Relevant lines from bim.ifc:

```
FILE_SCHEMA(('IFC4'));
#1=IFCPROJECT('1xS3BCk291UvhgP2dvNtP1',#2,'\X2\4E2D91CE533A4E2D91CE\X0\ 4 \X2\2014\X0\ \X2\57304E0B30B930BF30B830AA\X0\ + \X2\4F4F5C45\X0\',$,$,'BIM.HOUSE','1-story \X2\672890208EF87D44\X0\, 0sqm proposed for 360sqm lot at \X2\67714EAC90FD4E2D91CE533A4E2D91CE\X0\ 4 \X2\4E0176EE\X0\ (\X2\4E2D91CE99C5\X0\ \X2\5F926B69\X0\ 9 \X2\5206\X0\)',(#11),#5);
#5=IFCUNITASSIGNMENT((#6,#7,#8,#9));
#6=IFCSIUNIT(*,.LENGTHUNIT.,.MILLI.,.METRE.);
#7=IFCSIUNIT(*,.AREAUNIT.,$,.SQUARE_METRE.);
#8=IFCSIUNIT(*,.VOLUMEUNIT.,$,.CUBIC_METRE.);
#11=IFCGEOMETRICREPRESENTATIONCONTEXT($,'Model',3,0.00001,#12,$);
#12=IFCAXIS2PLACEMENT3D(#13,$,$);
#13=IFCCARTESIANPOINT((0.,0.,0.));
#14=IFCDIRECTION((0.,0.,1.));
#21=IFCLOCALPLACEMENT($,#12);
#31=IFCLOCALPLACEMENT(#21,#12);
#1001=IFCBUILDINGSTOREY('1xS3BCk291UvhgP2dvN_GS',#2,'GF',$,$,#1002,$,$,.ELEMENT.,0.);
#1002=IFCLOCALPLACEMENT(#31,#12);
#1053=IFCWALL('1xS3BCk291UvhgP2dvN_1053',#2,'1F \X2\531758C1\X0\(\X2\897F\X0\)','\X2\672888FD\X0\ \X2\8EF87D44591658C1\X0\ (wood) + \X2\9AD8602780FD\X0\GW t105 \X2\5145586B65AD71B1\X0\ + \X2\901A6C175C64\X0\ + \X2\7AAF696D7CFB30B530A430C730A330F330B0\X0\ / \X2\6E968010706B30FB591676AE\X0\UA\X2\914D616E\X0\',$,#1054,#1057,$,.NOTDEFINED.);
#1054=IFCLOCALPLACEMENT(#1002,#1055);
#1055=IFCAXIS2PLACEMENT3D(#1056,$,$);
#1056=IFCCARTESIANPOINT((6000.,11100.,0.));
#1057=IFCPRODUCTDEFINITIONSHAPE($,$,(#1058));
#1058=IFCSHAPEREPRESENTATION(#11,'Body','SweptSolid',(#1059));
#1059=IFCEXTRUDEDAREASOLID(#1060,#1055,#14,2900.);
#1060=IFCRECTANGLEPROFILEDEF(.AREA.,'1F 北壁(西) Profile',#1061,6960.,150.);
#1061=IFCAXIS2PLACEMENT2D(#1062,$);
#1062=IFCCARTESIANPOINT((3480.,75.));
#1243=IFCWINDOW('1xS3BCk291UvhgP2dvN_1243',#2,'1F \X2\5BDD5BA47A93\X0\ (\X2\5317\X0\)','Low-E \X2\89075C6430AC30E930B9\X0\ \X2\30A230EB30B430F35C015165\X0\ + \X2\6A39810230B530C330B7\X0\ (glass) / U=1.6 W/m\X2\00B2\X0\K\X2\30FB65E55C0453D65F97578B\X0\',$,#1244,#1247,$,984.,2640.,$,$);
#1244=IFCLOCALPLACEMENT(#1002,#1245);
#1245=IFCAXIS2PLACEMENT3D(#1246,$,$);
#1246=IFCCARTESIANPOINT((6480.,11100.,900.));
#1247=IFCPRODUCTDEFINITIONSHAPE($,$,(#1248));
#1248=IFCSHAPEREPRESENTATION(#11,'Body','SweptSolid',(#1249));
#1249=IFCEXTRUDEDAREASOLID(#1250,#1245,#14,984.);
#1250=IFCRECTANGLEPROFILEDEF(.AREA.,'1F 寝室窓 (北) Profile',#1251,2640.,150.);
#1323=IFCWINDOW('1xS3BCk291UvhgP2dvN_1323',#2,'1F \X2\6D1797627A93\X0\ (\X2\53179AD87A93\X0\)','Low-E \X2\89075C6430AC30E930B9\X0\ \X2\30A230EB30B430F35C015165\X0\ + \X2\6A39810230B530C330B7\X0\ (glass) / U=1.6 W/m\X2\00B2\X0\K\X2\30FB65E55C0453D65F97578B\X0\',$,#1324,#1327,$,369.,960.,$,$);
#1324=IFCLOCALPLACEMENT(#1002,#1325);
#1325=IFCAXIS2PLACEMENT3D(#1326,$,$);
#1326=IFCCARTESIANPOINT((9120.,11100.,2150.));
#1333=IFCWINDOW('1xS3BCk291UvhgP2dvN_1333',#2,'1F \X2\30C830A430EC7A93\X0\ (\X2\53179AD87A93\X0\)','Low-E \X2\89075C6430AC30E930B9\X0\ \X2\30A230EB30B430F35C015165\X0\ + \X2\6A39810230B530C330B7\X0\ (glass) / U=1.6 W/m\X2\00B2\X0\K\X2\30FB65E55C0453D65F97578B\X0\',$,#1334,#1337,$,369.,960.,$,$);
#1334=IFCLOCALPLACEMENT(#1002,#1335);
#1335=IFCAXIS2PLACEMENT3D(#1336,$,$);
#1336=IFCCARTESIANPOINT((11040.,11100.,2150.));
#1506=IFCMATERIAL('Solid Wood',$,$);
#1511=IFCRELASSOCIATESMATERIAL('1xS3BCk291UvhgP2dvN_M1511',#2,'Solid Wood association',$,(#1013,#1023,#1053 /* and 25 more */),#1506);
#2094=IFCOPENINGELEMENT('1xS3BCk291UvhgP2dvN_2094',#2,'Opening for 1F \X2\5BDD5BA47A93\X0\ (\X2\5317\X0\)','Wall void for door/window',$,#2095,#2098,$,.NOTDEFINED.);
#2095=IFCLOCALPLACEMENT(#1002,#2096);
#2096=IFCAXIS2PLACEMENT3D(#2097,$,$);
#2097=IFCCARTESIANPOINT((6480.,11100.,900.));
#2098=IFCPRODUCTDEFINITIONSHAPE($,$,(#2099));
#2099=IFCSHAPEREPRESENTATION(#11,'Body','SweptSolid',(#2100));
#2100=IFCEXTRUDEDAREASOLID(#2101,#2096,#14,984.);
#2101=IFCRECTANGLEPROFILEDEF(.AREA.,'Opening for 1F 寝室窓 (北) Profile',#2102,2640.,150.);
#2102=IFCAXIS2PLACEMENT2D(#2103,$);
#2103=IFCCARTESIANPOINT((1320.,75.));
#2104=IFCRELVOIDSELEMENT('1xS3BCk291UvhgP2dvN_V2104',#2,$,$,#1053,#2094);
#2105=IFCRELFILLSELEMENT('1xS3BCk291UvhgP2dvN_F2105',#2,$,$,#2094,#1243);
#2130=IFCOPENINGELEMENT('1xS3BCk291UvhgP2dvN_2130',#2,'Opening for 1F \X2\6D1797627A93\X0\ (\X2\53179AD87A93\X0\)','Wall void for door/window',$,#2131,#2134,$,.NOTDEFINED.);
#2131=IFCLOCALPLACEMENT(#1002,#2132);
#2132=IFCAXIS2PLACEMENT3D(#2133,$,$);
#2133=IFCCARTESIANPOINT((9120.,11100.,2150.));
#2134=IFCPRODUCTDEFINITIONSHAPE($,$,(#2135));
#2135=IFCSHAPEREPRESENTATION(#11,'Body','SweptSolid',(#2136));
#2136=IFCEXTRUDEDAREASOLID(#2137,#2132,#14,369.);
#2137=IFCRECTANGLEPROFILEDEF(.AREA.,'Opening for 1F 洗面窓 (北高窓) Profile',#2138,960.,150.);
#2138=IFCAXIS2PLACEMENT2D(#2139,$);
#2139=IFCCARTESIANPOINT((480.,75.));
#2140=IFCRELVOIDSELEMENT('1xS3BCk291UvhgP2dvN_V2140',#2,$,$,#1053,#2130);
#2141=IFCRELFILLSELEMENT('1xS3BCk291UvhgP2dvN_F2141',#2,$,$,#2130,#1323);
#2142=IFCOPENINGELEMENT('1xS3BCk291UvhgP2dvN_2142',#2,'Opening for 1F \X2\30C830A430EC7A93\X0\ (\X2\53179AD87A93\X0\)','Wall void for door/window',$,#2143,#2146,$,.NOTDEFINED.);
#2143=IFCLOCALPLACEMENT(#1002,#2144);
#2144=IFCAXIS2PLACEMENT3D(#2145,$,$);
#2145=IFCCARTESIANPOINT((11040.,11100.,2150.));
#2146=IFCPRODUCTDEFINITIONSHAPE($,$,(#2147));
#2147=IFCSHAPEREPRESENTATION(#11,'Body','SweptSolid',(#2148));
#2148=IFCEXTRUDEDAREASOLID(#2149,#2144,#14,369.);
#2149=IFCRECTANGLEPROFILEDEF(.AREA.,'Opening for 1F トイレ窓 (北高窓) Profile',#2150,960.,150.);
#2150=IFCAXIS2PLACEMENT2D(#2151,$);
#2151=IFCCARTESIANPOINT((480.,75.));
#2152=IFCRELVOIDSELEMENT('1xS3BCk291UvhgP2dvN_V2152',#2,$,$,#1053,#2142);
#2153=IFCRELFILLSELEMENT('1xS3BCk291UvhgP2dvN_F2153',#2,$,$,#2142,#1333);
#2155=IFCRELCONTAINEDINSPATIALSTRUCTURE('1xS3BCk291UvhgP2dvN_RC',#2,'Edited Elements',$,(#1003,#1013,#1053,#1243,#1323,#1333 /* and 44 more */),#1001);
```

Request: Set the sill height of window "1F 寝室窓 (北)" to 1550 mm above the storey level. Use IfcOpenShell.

```python
import numpy as np
import ifcopenshell
import ifcopenshell.api.geometry
import ifcopenshell.geom
import ifcopenshell.util.element
import ifcopenshell.util.placement
import ifcopenshell.util.shape
import ifcopenshell.util.unit

model = ifcopenshell.open("bim.ifc")
unit_scale = ifcopenshell.util.unit.calculate_unit_scale(model)

window = model.by_guid("1xS3BCk291UvhgP2dvN_1243")
opening = window.FillsVoids[0].RelatingOpeningElement
storey = ifcopenshell.util.element.get_container(window, ifc_class="IfcBuildingStorey")
level = ifcopenshell.util.placement.get_local_placement(storey.ObjectPlacement)[2, 3]

# The opening's origin need not be at the sill, so measure its lowest point.
shape = ifcopenshell.geom.create_shape(ifcopenshell.geom.settings(), opening)
bottom = ifcopenshell.util.shape.get_shape_bottom_elevation(shape, shape.geometry) / unit_scale
dz = level + 1.55 / unit_scale - bottom

shift = np.array([0.0, 0.0, dz])
# The window is not placed relative to its opening, so move both.
for product in (opening, window):
    matrix = ifcopenshell.util.placement.get_local_placement(product.ObjectPlacement)
    matrix[:3, 3] += shift
    ifcopenshell.api.geometry.edit_object_placement(model, product=product, matrix=matrix, is_si=False)

print(f"moved by {dz * unit_scale:+.3f} m")

model.write("bim_rev.ifc")
```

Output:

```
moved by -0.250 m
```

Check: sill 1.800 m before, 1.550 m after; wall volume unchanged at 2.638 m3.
